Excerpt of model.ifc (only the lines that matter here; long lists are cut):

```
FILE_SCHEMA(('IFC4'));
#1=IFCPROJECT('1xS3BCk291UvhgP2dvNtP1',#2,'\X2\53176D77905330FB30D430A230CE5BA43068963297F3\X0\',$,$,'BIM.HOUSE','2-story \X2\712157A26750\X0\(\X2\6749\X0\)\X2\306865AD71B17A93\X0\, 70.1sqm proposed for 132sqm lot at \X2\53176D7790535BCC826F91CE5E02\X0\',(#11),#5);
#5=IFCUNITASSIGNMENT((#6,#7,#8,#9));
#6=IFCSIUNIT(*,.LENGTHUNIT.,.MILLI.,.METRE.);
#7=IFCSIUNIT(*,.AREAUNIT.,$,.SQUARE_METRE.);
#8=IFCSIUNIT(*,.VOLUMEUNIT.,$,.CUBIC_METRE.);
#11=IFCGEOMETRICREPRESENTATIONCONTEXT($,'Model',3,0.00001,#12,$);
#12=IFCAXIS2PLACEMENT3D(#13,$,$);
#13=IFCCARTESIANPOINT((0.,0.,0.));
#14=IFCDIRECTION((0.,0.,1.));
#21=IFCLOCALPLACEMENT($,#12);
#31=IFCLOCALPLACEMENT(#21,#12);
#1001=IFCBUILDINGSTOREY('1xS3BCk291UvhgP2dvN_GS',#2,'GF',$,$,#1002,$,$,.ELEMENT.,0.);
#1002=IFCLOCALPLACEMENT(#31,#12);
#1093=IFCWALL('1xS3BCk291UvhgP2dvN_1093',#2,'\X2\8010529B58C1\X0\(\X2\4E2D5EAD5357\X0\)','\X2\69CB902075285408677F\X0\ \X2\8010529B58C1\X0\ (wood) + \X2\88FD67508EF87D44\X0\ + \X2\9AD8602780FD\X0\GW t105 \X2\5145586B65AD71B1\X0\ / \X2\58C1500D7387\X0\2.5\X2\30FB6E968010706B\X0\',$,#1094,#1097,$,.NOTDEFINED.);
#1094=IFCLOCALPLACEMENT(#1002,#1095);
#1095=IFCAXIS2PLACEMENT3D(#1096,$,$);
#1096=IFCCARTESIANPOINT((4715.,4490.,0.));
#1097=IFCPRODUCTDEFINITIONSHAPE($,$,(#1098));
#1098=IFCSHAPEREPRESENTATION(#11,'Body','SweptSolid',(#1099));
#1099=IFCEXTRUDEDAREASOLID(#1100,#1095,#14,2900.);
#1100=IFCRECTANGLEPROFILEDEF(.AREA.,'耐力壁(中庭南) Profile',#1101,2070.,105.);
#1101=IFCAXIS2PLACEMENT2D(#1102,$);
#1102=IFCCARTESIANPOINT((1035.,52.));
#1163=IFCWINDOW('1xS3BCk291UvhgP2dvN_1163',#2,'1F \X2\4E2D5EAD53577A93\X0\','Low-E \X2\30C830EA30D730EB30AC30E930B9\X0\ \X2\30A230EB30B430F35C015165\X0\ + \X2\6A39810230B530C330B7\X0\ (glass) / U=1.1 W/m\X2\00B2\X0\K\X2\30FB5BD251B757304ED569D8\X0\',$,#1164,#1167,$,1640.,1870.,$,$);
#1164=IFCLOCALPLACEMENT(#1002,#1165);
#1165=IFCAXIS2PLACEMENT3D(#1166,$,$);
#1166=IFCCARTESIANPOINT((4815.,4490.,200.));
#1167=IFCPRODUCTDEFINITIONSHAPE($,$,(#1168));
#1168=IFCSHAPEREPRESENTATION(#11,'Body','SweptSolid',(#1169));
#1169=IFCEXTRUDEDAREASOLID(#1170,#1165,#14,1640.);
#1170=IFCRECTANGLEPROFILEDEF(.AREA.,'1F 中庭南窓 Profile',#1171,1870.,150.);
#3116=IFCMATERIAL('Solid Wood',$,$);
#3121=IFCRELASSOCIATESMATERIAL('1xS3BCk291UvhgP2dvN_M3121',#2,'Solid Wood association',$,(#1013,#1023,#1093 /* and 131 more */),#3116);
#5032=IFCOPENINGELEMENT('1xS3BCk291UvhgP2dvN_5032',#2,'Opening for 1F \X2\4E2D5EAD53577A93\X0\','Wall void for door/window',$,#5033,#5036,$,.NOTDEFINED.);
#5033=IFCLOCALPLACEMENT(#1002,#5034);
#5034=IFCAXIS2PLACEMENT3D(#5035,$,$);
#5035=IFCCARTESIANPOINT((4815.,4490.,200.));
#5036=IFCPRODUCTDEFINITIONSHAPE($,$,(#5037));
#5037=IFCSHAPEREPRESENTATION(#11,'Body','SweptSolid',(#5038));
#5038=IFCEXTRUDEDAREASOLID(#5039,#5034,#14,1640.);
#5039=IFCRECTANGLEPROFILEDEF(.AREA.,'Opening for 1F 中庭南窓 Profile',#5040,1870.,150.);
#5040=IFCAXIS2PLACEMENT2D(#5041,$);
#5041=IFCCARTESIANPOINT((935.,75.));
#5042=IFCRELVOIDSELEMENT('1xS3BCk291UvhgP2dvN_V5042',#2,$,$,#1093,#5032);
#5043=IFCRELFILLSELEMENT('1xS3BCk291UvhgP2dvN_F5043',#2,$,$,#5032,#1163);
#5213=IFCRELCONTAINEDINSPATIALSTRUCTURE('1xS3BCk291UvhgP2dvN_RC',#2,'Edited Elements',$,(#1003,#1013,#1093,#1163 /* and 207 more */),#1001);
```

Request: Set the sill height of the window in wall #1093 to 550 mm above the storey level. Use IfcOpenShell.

```python
import numpy as np
import ifcopenshell
import ifcopenshell.api.geometry
import ifcopenshell.geom
import ifcopenshell.util.element
import ifcopenshell.util.placement
import ifcopenshell.util.shape
import ifcopenshell.util.unit

model = ifcopenshell.open("model.ifc")
unit_scale = ifcopenshell.util.unit.calculate_unit_scale(model)

window = model.by_guid("1xS3BCk291UvhgP2dvN_1163")
opening = window.FillsVoids[0].RelatingOpeningElement
storey = ifcopenshell.util.element.get_container(window, ifc_class="IfcBuildingStorey")
level = ifcopenshell.util.placement.get_local_placement(storey.ObjectPlacement)[2, 3]

# The opening's origin need not be at the sill, so measure its lowest point.
shape = ifcopenshell.geom.create_shape(ifcopenshell.geom.settings(), opening)
bottom = ifcopenshell.util.shape.get_shape_bottom_elevation(shape, shape.geometry) / unit_scale
dz = level + 0.55 / unit_scale - bottom

shift = np.array([0.0, 0.0, dz])
# The window is not placed relative to its opening, so move both.
for product in (opening, window):
    matrix = ifcopenshell.util.placement.get_local_placement(product.ObjectPlacement)
    matrix[:3, 3] += shift
    ifcopenshell.api.geometry.edit_object_placement(model, product=product, matrix=matrix, is_si=False)

print(f"moved by {dz * unit_scale:+.3f} m")

model.write("model_rev.ifc")
```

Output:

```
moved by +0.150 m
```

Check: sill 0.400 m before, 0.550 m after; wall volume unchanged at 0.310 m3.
